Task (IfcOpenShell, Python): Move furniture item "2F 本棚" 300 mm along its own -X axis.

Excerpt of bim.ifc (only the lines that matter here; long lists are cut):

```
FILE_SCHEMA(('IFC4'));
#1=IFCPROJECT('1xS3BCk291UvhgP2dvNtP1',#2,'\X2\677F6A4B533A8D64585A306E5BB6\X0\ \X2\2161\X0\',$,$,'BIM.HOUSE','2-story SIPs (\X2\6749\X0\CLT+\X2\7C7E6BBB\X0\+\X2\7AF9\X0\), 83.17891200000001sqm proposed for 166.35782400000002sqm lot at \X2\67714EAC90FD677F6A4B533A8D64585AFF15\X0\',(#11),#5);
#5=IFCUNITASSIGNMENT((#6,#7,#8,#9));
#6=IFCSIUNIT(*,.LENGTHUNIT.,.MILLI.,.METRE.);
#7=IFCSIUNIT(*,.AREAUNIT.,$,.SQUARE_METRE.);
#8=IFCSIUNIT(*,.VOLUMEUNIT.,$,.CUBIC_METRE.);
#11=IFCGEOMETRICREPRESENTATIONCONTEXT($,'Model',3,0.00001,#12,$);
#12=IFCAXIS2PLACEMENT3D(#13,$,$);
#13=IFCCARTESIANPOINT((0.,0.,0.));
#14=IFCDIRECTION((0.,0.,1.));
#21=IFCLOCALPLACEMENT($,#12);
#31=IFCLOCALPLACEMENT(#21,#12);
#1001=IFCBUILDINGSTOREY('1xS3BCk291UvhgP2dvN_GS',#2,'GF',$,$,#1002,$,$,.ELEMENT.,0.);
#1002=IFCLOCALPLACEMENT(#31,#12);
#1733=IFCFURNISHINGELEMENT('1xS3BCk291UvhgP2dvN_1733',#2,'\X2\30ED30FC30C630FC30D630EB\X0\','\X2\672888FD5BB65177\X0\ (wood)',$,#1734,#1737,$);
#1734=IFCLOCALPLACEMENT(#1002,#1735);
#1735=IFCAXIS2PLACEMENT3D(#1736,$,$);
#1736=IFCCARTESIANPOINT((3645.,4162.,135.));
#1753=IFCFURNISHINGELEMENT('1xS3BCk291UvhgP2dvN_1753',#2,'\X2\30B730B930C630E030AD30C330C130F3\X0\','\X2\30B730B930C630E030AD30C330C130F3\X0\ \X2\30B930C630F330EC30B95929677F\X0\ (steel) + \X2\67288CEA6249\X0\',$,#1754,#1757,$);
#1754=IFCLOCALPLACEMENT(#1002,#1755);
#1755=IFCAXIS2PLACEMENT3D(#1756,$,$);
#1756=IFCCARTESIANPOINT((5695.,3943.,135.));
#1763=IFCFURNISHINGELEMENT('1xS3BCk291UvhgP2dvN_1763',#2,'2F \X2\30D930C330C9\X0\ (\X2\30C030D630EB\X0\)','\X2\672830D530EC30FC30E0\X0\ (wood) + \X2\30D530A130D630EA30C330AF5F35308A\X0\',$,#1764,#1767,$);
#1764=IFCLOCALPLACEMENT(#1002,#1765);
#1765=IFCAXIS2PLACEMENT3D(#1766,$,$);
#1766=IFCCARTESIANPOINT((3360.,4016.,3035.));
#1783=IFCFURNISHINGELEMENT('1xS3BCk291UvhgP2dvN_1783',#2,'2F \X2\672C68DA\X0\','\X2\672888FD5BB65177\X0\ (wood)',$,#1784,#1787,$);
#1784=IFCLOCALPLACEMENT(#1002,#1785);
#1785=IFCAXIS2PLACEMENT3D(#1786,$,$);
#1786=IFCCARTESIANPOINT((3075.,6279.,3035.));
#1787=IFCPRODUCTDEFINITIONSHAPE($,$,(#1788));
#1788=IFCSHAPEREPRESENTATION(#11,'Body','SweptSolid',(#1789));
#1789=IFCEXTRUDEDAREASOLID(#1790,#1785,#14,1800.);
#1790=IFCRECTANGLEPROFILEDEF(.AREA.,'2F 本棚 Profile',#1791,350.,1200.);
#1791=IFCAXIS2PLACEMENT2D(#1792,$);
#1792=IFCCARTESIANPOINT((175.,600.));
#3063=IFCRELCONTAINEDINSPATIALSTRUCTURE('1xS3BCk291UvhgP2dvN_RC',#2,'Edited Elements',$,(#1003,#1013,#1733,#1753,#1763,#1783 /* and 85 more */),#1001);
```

```python
import ifcopenshell
import ifcopenshell.api.geometry
import ifcopenshell.util.placement
import ifcopenshell.util.unit

model = ifcopenshell.open("bim.ifc")
unit_scale = ifcopenshell.util.unit.calculate_unit_scale(model)

item = model.by_guid("1xS3BCk291UvhgP2dvN_1783")
matrix = ifcopenshell.util.placement.get_local_placement(item.ObjectPlacement)
matrix[:3, 3] -= matrix[:3, 0] * 0.3 / unit_scale
ifcopenshell.api.geometry.edit_object_placement(model, product=item, matrix=matrix, is_si=False)

print(ifcopenshell.util.placement.get_local_placement(item.ObjectPlacement).round(3) + 0.0)

model.write("bim_v2.ifc")
```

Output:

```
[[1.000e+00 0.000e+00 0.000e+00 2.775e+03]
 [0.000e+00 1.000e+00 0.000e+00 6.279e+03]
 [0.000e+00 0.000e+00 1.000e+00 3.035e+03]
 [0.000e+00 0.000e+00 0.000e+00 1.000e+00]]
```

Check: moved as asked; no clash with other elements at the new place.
